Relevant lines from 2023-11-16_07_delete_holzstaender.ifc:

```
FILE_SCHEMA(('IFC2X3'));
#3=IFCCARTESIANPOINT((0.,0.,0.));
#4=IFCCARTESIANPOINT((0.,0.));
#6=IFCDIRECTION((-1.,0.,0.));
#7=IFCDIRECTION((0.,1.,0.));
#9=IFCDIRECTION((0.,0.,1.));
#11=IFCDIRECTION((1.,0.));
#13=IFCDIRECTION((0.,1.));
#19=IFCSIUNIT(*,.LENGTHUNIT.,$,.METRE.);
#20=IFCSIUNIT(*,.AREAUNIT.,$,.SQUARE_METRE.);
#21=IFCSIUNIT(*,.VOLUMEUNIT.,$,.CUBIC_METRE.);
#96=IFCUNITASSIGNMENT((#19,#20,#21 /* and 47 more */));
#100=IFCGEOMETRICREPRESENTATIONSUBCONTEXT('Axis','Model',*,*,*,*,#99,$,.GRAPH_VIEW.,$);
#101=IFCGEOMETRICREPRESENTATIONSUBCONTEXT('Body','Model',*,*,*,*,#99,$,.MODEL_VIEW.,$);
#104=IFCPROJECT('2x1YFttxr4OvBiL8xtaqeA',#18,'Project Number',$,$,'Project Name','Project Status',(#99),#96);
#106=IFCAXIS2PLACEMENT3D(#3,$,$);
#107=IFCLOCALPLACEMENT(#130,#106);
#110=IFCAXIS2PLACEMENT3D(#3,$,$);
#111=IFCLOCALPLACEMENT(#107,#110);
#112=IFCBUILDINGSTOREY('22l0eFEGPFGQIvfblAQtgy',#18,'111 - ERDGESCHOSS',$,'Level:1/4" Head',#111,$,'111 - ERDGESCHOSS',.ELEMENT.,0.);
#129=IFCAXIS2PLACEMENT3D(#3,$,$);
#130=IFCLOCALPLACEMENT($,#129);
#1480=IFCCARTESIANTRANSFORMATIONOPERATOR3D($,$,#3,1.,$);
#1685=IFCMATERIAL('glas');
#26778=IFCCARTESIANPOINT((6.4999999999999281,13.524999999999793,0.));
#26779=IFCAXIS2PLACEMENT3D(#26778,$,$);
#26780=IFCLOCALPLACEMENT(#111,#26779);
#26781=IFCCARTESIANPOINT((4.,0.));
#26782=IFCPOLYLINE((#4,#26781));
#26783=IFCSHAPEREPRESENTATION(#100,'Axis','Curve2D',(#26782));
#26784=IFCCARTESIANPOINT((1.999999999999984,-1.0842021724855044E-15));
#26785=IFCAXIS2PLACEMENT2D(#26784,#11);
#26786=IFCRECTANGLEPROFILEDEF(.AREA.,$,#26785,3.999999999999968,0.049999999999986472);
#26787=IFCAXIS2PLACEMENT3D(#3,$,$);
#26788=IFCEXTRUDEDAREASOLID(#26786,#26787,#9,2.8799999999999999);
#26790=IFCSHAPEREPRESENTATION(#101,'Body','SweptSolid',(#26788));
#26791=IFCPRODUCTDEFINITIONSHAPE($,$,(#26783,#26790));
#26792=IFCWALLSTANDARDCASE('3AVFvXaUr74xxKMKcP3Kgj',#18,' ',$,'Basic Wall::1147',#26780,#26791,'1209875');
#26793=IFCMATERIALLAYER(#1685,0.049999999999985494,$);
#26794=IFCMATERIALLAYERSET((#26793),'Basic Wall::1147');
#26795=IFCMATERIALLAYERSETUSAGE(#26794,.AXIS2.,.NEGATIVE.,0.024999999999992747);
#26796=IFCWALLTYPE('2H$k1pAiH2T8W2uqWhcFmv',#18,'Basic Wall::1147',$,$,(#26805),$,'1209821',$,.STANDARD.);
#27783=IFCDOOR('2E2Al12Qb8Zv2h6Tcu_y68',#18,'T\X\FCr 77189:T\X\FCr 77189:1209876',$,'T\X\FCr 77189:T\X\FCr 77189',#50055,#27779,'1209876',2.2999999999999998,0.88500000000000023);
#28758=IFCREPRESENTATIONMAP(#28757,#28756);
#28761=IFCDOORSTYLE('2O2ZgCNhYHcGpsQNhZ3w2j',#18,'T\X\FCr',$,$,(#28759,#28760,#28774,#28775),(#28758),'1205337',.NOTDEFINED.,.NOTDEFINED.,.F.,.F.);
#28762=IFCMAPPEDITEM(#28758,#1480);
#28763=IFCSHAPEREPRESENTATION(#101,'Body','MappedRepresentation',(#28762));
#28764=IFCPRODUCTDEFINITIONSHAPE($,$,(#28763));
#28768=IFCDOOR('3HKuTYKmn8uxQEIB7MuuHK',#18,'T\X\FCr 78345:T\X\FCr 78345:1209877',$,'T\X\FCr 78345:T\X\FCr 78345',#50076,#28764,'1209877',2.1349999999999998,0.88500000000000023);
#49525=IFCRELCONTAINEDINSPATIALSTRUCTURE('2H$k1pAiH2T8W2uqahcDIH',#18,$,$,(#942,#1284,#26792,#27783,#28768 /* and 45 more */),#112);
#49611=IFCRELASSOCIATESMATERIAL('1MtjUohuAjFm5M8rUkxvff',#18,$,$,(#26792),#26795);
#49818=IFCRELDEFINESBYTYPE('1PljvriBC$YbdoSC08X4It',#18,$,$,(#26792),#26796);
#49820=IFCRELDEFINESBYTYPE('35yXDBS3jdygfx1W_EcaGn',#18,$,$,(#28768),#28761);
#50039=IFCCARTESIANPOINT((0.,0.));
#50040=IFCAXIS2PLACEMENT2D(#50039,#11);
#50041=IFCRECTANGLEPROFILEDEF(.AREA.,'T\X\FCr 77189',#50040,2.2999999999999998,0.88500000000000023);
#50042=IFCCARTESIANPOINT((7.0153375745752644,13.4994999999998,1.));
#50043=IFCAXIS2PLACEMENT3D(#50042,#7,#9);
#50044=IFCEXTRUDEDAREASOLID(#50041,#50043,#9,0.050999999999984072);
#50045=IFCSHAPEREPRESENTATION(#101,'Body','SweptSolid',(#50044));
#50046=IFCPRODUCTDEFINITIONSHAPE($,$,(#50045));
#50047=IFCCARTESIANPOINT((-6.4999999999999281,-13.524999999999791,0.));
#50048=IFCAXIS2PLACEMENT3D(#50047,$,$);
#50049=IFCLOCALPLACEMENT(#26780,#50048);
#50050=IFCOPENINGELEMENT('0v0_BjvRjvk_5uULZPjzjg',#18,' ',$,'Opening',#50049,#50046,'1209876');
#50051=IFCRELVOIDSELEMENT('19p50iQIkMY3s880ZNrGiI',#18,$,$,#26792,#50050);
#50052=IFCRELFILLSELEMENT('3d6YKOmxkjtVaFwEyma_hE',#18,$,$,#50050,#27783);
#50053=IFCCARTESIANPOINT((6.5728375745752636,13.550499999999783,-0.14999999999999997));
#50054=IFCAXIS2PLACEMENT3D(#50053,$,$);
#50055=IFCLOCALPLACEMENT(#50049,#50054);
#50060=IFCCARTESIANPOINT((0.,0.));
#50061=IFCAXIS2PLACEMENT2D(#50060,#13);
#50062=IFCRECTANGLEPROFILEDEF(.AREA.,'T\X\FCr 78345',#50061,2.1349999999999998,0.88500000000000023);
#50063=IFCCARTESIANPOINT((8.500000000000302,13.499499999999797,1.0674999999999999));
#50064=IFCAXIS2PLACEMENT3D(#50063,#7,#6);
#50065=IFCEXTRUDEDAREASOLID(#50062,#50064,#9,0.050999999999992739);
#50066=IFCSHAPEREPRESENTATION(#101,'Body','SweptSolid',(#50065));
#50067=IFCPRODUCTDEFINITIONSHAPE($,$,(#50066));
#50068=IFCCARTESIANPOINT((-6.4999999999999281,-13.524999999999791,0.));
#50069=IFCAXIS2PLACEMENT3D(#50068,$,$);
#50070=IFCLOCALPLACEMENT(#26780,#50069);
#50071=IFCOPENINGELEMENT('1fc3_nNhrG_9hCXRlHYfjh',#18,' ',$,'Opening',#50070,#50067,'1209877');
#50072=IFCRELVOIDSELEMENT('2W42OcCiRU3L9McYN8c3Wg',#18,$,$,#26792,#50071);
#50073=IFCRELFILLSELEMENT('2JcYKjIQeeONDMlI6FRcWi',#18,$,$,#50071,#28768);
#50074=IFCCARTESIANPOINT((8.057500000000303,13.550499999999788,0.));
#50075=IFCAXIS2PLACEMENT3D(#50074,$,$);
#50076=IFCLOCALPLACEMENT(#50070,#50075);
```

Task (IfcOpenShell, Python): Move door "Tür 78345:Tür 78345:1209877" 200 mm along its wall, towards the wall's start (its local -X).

```python
import ifcopenshell
import ifcopenshell.api.geometry
import ifcopenshell.util.placement

model = ifcopenshell.open("2023-11-16_07_delete_holzstaender.ifc")

door = model.by_id(28768)
opening = door.FillsVoids[0].RelatingOpeningElement
wall = opening.VoidsElements[0].RelatingBuildingElement

wall_matrix = ifcopenshell.util.placement.get_local_placement(wall.ObjectPlacement)
shift = wall_matrix[:3, 0] * -0.2
before = ifcopenshell.util.placement.get_local_placement(door.ObjectPlacement)[:3, 3].copy()

# The door is placed relative to its opening, so it follows when the opening moves.
matrix = ifcopenshell.util.placement.get_local_placement(opening.ObjectPlacement)
matrix[:3, 3] += shift
ifcopenshell.api.geometry.edit_object_placement(
    model, product=opening, matrix=matrix, is_si=False, should_transform_children=True
)

after = ifcopenshell.util.placement.get_local_placement(door.ObjectPlacement)[:3, 3]
print("door moved by", (after - before).round(3) + 0.0)

model.write("2023-11-16_07_delete_holzstaender_edited.ifc")
```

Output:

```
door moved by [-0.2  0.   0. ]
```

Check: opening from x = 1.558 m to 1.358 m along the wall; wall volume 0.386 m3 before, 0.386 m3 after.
